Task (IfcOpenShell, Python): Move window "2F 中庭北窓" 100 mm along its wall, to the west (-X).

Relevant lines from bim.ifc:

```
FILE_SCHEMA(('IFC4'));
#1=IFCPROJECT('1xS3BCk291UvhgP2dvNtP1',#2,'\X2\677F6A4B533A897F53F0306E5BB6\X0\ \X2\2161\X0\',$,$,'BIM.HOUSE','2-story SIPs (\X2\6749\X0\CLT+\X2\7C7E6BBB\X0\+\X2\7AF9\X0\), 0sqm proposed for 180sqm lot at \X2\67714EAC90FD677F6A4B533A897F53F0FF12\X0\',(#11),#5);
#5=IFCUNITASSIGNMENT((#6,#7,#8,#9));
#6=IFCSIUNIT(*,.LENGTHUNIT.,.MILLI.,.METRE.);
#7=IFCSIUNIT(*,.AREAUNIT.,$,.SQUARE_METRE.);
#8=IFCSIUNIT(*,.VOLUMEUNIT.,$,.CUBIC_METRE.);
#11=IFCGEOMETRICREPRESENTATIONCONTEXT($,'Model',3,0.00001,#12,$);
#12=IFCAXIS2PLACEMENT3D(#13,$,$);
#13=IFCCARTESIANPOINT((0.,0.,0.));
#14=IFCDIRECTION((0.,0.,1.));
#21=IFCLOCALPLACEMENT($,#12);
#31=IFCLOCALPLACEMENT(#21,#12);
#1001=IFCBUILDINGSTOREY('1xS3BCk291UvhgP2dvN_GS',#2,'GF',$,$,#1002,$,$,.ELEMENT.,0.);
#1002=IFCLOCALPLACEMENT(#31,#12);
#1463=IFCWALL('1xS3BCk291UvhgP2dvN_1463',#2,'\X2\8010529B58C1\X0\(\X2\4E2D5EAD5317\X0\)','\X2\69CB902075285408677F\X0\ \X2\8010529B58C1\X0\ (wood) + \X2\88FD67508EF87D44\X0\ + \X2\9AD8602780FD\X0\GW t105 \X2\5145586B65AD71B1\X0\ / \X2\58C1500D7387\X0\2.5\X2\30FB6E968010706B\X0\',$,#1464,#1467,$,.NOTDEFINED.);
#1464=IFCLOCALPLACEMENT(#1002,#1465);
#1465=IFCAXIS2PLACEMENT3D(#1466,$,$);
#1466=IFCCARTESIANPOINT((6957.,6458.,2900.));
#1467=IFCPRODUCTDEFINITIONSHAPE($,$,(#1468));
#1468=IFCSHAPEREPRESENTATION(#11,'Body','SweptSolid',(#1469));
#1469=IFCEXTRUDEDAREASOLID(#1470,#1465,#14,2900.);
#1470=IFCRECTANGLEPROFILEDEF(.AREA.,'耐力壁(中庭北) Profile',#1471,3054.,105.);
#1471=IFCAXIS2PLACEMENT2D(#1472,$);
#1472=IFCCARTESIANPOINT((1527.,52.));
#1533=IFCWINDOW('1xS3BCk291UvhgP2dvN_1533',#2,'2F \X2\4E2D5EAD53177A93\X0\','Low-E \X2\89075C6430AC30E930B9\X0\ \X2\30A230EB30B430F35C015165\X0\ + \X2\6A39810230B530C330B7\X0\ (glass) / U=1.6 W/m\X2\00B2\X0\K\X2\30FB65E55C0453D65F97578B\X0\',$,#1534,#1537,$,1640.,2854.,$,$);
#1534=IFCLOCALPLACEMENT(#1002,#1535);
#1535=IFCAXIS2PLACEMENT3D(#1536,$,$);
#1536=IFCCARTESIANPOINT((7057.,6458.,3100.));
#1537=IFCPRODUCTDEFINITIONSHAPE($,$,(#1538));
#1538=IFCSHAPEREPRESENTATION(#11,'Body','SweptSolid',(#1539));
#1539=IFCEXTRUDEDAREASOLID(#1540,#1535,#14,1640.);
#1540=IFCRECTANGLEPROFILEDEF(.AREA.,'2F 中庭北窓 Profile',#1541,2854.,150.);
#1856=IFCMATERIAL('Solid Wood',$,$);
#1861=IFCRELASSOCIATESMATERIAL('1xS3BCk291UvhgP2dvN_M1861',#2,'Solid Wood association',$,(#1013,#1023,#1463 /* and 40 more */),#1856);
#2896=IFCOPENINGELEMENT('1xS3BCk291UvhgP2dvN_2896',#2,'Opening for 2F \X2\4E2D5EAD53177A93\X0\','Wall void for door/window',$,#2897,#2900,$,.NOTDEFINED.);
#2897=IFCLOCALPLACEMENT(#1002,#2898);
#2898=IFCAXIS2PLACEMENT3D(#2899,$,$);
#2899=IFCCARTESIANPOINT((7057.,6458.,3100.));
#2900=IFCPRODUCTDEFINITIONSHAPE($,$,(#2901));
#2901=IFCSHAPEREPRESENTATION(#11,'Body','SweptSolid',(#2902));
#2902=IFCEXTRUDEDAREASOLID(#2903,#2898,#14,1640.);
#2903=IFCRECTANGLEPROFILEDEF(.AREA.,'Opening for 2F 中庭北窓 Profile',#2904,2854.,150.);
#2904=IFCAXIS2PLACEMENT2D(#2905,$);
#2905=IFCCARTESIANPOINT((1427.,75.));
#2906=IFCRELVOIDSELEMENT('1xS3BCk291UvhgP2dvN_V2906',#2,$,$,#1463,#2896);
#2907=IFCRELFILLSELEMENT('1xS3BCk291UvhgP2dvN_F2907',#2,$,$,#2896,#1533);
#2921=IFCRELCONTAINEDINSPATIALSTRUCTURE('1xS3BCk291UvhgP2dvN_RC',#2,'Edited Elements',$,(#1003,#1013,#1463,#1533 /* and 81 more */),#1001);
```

```python
import ifcopenshell
import ifcopenshell.api.geometry
import ifcopenshell.util.placement

model = ifcopenshell.open("bim.ifc")

window = model.by_id(1533)
opening = window.FillsVoids[0].RelatingOpeningElement
wall = opening.VoidsElements[0].RelatingBuildingElement

wall_matrix = ifcopenshell.util.placement.get_local_placement(wall.ObjectPlacement)
shift = wall_matrix[:3, 0] * -100.0
before = ifcopenshell.util.placement.get_local_placement(window.ObjectPlacement)[:3, 3].copy()

# The window is not placed relative to its opening, so move both.
for product in (opening, window):
    matrix = ifcopenshell.util.placement.get_local_placement(product.ObjectPlacement)
    matrix[:3, 3] += shift
    ifcopenshell.api.geometry.edit_object_placement(model, product=product, matrix=matrix, is_si=False)

after = ifcopenshell.util.placement.get_local_placement(window.ObjectPlacement)[:3, 3]
print("window moved by", (after - before).round(3) + 0.0)

model.write("bim_updated.ifc")
```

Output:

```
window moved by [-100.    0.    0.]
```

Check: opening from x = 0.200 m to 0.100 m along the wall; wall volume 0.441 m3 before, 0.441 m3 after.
